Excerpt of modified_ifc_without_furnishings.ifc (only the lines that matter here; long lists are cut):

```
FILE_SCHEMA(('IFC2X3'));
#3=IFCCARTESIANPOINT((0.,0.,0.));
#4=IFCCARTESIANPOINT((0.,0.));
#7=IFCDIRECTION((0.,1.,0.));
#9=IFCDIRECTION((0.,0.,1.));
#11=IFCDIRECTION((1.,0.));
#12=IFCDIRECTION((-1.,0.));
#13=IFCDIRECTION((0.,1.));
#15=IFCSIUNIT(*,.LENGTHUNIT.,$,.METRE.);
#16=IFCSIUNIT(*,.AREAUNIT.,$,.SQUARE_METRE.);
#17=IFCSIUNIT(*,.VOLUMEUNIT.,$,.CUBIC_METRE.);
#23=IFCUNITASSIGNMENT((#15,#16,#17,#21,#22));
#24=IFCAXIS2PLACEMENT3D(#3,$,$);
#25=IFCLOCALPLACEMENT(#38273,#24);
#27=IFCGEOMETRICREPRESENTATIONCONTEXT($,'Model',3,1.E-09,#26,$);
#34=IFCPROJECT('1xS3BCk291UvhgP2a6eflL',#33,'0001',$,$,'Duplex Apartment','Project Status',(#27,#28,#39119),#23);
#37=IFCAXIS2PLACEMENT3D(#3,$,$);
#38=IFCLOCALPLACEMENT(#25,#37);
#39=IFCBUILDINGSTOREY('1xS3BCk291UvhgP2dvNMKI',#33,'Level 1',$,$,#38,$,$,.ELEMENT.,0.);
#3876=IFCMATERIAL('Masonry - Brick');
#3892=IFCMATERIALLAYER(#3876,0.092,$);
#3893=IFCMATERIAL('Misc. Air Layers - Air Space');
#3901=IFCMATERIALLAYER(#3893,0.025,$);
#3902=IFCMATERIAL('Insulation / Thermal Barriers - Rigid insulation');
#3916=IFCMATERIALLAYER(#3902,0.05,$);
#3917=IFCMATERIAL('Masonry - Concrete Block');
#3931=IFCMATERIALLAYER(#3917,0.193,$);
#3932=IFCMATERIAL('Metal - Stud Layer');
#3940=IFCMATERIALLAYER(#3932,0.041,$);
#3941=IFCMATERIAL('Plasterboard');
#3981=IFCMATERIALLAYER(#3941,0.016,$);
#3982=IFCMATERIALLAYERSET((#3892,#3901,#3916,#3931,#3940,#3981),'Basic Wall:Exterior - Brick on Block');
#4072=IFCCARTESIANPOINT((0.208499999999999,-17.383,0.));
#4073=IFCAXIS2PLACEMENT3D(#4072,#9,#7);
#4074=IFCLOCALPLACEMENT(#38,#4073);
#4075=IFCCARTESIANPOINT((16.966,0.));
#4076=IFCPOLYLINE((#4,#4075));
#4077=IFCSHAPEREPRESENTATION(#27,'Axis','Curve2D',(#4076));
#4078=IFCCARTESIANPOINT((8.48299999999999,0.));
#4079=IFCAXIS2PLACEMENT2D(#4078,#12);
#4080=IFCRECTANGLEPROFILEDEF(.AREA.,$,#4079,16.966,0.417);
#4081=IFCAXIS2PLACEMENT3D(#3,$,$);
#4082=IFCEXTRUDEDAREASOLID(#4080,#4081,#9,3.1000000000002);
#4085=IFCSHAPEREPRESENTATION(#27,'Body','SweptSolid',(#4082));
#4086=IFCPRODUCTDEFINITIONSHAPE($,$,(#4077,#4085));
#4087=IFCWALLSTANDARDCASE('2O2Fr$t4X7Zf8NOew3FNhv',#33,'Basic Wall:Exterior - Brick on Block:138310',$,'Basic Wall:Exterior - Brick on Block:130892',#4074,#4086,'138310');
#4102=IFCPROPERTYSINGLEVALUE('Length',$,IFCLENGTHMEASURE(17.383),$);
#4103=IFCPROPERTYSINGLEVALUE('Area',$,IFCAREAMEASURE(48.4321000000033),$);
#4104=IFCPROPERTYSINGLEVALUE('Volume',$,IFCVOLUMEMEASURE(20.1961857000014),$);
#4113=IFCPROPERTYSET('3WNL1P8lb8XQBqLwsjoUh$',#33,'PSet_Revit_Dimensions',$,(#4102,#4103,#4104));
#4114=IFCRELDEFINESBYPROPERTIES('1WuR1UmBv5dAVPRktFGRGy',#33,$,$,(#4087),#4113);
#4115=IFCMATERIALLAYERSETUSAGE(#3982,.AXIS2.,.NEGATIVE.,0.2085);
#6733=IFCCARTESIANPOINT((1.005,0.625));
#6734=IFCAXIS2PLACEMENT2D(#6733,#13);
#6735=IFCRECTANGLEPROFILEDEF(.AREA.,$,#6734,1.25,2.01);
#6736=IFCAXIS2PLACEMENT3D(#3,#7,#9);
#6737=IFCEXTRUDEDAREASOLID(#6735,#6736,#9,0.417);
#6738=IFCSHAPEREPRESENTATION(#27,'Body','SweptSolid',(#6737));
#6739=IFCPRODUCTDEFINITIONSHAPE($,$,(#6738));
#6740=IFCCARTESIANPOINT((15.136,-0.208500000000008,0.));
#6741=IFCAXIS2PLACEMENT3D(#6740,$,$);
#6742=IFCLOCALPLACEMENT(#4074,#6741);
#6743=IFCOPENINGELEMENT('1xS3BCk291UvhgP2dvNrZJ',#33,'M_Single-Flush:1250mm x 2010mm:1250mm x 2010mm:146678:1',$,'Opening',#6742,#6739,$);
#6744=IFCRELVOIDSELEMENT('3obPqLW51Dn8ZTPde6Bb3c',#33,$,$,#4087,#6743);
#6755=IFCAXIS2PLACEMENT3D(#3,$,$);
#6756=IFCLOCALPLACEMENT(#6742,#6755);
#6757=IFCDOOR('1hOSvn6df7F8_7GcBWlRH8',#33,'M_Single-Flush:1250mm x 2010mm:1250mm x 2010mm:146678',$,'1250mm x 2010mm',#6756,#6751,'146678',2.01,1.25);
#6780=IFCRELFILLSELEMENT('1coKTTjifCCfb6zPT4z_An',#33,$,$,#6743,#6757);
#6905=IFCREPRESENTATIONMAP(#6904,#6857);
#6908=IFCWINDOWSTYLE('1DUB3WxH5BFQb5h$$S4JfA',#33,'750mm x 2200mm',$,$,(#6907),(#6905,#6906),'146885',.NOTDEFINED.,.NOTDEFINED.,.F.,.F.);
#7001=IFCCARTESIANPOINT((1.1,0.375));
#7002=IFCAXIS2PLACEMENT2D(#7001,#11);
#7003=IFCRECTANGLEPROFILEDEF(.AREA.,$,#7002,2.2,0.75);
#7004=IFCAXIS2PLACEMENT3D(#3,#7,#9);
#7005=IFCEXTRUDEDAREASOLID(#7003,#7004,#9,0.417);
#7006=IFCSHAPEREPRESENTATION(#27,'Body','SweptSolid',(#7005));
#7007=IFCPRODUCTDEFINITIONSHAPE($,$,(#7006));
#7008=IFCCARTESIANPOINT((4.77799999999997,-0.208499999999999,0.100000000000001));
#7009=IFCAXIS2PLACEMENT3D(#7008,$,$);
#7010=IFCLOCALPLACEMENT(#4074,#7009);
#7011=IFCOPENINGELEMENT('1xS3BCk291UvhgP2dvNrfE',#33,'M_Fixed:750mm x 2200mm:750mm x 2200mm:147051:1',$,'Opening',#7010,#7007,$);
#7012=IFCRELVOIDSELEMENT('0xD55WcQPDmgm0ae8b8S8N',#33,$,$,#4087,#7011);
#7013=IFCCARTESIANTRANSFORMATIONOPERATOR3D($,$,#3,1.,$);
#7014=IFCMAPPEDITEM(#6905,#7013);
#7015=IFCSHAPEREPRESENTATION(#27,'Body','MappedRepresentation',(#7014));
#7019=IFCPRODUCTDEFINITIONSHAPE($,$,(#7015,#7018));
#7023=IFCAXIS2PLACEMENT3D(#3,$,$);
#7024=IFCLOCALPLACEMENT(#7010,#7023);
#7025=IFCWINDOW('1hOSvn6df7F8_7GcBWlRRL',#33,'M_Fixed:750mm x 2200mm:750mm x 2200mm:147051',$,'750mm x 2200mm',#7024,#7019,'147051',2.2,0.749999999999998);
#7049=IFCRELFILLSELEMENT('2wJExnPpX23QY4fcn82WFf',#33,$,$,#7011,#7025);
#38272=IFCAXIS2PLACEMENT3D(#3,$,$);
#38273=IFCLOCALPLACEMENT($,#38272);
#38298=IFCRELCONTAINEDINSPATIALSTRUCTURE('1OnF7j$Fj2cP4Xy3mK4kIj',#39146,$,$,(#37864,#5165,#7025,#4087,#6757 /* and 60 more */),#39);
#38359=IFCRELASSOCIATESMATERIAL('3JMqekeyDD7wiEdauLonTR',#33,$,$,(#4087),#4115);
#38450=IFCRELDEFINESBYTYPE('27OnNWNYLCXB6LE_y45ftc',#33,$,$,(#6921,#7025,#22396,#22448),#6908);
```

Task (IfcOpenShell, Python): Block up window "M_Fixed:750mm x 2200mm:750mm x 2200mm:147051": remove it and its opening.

```python
import ifcopenshell
import ifcopenshell.api.feature
import ifcopenshell.api.pset
import ifcopenshell.api.root
import ifcopenshell.geom
import ifcopenshell.util.element
import ifcopenshell.util.shape
import ifcopenshell.util.unit

model = ifcopenshell.open("modified_ifc_without_furnishings.ifc")
area_scale = ifcopenshell.util.unit.calculate_unit_scale(model, "AREAUNIT")
volume_scale = ifcopenshell.util.unit.calculate_unit_scale(model, "VOLUMEUNIT")
settings = ifcopenshell.geom.settings()


def volume(element):
    """Net volume in cubic metres, openings subtracted."""
    shape = ifcopenshell.geom.create_shape(settings, element)
    return ifcopenshell.util.shape.get_volume(shape.geometry)


window = model.by_guid("1hOSvn6df7F8_7GcBWlRRL")
opening = window.FillsVoids[0].RelatingOpeningElement
wall = opening.VoidsElements[0].RelatingBuildingElement
before = volume(wall)

ifcopenshell.api.root.remove_product(model, product=window)
ifcopenshell.api.feature.remove_feature(model, feature=opening)

after = volume(wall)
thickness = 0.417  # wall thickness in metres

# Update the wall's stored quantities.
pset = model.by_id(ifcopenshell.util.element.get_pset(wall, "PSet_Revit_Dimensions", should_inherit=False)["id"])
ifcopenshell.api.pset.edit_pset(model, pset=pset, properties={
    "Area": model.create_entity("IfcAreaMeasure", after / thickness / area_scale),
    "Volume": model.create_entity("IfcVolumeMeasure", after / volume_scale),
})

print(f"wall volume {before:.3f} -> {after:.3f} m3")

model.write("modified_ifc_without_furnishings_edited.ifc")
```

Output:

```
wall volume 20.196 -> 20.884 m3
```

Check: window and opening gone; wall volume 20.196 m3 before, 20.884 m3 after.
